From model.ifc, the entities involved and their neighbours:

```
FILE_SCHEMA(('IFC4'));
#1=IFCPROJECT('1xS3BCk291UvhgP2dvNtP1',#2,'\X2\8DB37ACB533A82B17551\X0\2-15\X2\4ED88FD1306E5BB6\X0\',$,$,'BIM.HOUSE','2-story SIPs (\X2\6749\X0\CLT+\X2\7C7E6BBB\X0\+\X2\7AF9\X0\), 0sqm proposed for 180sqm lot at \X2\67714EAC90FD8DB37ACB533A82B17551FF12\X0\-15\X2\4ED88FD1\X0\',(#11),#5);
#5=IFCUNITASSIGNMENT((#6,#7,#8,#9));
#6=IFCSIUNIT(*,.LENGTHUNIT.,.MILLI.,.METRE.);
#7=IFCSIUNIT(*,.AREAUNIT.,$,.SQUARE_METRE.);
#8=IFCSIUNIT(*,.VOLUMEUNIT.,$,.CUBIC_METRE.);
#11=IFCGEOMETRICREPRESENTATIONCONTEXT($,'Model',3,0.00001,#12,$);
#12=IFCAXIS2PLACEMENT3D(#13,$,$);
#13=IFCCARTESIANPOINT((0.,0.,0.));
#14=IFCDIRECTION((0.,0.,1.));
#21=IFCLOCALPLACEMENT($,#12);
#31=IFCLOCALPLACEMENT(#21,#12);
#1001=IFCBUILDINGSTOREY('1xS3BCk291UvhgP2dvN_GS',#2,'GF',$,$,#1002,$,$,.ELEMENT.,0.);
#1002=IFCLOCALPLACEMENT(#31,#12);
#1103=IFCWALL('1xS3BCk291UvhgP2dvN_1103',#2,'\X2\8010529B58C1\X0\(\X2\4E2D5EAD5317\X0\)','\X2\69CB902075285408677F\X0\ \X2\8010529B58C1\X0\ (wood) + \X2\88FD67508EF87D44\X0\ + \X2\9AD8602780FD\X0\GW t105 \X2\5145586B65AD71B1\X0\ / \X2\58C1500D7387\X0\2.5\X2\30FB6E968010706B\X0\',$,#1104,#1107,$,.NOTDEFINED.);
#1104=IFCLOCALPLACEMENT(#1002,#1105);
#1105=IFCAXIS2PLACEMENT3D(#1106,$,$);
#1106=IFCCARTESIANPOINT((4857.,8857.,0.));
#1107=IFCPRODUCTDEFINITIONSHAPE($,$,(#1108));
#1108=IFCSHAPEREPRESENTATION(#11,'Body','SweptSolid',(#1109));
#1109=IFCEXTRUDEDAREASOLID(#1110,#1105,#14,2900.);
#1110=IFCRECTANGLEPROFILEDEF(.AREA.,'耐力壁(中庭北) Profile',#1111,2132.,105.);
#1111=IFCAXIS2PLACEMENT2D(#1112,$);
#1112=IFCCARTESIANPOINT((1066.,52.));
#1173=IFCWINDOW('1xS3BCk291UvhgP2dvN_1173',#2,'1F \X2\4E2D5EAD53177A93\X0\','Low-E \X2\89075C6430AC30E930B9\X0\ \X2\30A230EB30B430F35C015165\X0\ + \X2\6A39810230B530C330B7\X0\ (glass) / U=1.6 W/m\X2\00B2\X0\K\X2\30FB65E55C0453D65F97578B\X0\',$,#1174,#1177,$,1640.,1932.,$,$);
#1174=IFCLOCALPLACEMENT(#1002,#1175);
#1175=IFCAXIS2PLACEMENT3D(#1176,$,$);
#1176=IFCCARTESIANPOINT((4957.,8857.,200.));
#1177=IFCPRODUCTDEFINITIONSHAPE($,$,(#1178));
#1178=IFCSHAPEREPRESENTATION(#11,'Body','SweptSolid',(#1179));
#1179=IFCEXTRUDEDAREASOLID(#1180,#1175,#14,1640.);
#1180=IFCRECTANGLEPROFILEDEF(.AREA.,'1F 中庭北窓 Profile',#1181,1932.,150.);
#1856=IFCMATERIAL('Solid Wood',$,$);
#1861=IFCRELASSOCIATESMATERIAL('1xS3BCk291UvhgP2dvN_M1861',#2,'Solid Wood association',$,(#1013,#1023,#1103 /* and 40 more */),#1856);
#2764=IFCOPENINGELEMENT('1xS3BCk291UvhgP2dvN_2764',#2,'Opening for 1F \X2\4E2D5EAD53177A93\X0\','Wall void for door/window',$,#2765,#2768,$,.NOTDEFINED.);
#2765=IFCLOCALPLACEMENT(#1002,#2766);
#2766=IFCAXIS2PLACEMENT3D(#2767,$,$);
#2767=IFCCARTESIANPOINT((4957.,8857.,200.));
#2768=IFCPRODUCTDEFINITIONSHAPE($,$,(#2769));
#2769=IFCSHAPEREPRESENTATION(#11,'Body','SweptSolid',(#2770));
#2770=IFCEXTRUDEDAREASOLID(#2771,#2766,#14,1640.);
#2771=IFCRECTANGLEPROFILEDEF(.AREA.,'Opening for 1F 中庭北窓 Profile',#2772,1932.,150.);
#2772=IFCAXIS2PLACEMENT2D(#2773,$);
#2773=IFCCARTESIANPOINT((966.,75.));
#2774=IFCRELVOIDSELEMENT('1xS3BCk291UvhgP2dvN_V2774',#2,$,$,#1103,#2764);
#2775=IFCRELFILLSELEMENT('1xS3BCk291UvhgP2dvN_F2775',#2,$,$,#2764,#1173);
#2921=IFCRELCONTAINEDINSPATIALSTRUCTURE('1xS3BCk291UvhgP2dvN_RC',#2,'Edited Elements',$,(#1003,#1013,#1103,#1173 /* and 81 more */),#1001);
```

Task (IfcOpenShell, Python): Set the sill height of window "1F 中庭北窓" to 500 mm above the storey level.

```python
import numpy as np
import ifcopenshell
import ifcopenshell.api.geometry
import ifcopenshell.geom
import ifcopenshell.util.element
import ifcopenshell.util.placement
import ifcopenshell.util.shape
import ifcopenshell.util.unit

model = ifcopenshell.open("model.ifc")
unit_scale = ifcopenshell.util.unit.calculate_unit_scale(model)

window = model.by_guid("1xS3BCk291UvhgP2dvN_1173")
opening = window.FillsVoids[0].RelatingOpeningElement
storey = ifcopenshell.util.element.get_container(window, ifc_class="IfcBuildingStorey")
level = ifcopenshell.util.placement.get_local_placement(storey.ObjectPlacement)[2, 3]

# The opening's origin need not be at the sill, so measure its lowest point.
shape = ifcopenshell.geom.create_shape(ifcopenshell.geom.settings(), opening)
bottom = ifcopenshell.util.shape.get_shape_bottom_elevation(shape, shape.geometry) / unit_scale
dz = level + 0.5 / unit_scale - bottom

shift = np.array([0.0, 0.0, dz])
# The window is not placed relative to its opening, so move both.
for product in (opening, window):
    matrix = ifcopenshell.util.placement.get_local_placement(product.ObjectPlacement)
    matrix[:3, 3] += shift
    ifcopenshell.api.geometry.edit_object_placement(model, product=product, matrix=matrix, is_si=False)

print(f"moved by {dz * unit_scale:+.3f} m")

model.write("model-out.ifc")
```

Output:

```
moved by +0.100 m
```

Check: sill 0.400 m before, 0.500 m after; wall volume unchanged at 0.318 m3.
